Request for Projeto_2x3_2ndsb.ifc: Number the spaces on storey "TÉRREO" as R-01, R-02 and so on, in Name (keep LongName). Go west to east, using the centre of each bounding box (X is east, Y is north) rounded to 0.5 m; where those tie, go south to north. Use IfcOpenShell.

First a look at what the model holds.

```python
import ifcopenshell
import ifcopenshell.util.element
import ifcopenshell.util.placement

model = ifcopenshell.open("Projeto_2x3_2ndsb.ifc")
print(model.schema)
storey = next(s for s in model.by_type("IfcBuildingStorey") if s.Name == "TÉRREO")
spaces = [e for e in ifcopenshell.util.element.get_decomposition(storey) if e.is_a("IfcSpace")]
for e in sorted(spaces, key=lambda e: e.id()):
    origin = ifcopenshell.util.placement.get_local_placement(e.ObjectPlacement)[:3, 3]
    print(e.id(), e.Name, e.LongName, origin.round(2) + 0.0, sep=" | ")
```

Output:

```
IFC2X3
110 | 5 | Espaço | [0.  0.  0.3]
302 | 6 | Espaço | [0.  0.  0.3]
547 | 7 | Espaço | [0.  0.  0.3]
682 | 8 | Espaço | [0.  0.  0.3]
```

```python
import ifcopenshell
import ifcopenshell.geom
import ifcopenshell.util.element
import ifcopenshell.util.shape

model = ifcopenshell.open("Projeto_2x3_2ndsb.ifc")
settings = ifcopenshell.geom.settings()
settings.set("use-world-coords", True)


def centre(element):
    shape = ifcopenshell.geom.create_shape(settings, element)
    return ifcopenshell.util.shape.get_bbox_centroid(shape.geometry)


storey = next(s for s in model.by_type("IfcBuildingStorey") if s.Name == "TÉRREO")
spaces = [e for e in ifcopenshell.util.element.get_decomposition(storey) if e.is_a("IfcSpace")]

# Insertion points can sit at a corner or the storey origin, so sort by the geometry (in metres).
centres = {e: centre(e) for e in spaces}
spaces.sort(key=lambda e: (round(centres[e][0] / 0.5), centres[e][1]))

for i, e in enumerate(spaces, start=1):
    number = f"R-{i:02d}"
    e.Name = number
    print(e.id(), number)

model.write("Projeto_2x3_2ndsb-out.ifc")
```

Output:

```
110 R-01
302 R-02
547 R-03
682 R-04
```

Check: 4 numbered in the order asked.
